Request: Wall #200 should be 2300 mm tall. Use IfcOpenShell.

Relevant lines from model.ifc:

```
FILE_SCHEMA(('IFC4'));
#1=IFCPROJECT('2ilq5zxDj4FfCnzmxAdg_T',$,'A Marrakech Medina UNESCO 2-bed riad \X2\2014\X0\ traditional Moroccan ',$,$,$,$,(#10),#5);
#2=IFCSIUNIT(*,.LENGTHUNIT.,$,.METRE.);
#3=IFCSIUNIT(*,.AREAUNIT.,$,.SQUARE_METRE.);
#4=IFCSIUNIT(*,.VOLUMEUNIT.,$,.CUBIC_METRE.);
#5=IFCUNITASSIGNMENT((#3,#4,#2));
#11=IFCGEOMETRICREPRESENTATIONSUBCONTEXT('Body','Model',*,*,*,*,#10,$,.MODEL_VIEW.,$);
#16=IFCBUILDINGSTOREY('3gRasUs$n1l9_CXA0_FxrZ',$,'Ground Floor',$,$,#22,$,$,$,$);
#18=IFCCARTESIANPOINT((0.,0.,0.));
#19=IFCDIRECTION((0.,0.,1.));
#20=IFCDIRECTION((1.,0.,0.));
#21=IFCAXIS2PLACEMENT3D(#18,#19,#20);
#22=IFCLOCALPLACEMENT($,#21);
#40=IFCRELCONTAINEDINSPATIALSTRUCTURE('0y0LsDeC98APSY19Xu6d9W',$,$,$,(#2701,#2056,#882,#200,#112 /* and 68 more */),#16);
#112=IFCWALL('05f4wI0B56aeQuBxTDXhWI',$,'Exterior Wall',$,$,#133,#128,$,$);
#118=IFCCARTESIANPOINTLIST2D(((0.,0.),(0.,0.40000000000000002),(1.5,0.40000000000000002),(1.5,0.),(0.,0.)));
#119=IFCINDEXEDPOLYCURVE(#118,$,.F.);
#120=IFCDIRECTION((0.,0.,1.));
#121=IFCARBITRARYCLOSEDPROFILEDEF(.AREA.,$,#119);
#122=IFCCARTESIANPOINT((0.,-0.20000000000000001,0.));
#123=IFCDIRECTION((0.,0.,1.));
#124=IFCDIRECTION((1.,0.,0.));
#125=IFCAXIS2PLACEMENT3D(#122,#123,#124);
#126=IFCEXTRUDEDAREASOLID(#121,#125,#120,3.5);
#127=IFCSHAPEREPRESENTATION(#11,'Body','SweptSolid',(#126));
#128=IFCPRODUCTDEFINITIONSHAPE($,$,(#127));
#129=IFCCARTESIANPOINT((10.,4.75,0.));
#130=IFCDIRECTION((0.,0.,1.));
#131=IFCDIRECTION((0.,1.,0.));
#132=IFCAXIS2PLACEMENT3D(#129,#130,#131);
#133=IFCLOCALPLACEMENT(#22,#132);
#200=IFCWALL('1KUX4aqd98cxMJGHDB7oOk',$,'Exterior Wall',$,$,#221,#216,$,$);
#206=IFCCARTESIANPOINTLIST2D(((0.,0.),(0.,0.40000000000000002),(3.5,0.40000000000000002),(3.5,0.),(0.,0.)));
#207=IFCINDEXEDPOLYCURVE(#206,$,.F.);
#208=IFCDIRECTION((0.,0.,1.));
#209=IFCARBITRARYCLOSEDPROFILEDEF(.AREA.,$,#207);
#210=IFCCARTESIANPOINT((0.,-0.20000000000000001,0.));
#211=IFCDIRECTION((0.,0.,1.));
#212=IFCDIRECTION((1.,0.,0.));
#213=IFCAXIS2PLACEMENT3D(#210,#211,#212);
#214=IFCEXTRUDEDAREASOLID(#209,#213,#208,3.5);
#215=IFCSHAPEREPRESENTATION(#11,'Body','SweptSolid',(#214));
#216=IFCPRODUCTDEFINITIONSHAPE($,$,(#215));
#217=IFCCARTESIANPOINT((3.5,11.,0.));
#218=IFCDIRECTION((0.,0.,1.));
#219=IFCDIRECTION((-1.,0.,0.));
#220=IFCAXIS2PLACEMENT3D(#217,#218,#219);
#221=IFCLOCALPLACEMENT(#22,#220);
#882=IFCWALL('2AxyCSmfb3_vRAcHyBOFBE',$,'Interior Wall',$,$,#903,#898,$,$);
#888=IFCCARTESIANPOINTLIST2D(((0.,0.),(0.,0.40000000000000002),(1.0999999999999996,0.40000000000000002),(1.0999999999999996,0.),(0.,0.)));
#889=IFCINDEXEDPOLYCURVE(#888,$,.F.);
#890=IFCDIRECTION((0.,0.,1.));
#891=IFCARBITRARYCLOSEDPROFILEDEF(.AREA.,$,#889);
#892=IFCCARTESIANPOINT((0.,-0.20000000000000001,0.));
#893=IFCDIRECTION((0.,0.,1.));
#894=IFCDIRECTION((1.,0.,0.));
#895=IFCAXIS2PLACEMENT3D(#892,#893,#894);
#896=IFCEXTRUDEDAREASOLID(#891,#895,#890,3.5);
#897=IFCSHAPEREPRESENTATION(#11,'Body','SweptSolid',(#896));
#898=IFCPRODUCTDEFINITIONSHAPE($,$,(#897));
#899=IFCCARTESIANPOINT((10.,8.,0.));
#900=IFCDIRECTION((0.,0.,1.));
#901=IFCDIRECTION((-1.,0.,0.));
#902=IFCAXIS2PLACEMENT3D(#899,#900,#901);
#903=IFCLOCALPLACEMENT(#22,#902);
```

```python
import ifcopenshell
import ifcopenshell.geom
import ifcopenshell.util.representation
import ifcopenshell.util.shape
import ifcopenshell.util.unit

model = ifcopenshell.open("model.ifc")
unit_scale = ifcopenshell.util.unit.calculate_unit_scale(model)
settings = ifcopenshell.geom.settings()


def volume(element):
    """Net volume in cubic metres, openings subtracted."""
    shape = ifcopenshell.geom.create_shape(settings, element)
    return ifcopenshell.util.shape.get_volume(shape.geometry)


wall = model.by_guid("1KUX4aqd98cxMJGHDB7oOk")
before = volume(wall)

body = ifcopenshell.util.representation.get_representation(wall, "Model", "Body")
solid = body.Items[0]
old_height = solid.Depth
solid.Depth = 2.3 / unit_scale
after = volume(wall)

print(f"height {old_height:g} -> {solid.Depth:g}, volume {before:.3f} -> {after:.3f} m3")

model.write("model-out.ifc")
```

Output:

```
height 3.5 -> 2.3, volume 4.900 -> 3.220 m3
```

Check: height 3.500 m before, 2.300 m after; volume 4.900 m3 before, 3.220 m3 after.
